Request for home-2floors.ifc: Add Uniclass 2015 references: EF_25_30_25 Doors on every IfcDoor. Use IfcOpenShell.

First a look at what the model holds.

```python
import ifcopenshell

model = ifcopenshell.open("home-2floors.ifc")
print(model.schema)
print("classifications:", [c.Name for c in model.by_type("IfcClassification")])
for ifc_class in ("IfcDoor", "IfcRoof", "IfcStair", "IfcWall", "IfcWindow"):
    print(ifc_class, len(model.by_type(ifc_class)))
```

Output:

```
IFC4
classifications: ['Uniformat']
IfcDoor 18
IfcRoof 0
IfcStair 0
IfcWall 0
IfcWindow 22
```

```python
import ifcopenshell
import ifcopenshell.api.classification

model = ifcopenshell.open("home-2floors.ifc")

system = ifcopenshell.api.classification.add_classification(model, classification="Uniclass 2015")

codes = {
    "IfcDoor": ("EF_25_30_25", "Doors"),
}
for ifc_class, (code, name) in codes.items():
    products = model.by_type(ifc_class)
    ifcopenshell.api.classification.add_reference(
        model, products=products, classification=system, identification=code, name=name
    )
    print(code, len(products))

model.write("home-2floors_updated.ifc")
```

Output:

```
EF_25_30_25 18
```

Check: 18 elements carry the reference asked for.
